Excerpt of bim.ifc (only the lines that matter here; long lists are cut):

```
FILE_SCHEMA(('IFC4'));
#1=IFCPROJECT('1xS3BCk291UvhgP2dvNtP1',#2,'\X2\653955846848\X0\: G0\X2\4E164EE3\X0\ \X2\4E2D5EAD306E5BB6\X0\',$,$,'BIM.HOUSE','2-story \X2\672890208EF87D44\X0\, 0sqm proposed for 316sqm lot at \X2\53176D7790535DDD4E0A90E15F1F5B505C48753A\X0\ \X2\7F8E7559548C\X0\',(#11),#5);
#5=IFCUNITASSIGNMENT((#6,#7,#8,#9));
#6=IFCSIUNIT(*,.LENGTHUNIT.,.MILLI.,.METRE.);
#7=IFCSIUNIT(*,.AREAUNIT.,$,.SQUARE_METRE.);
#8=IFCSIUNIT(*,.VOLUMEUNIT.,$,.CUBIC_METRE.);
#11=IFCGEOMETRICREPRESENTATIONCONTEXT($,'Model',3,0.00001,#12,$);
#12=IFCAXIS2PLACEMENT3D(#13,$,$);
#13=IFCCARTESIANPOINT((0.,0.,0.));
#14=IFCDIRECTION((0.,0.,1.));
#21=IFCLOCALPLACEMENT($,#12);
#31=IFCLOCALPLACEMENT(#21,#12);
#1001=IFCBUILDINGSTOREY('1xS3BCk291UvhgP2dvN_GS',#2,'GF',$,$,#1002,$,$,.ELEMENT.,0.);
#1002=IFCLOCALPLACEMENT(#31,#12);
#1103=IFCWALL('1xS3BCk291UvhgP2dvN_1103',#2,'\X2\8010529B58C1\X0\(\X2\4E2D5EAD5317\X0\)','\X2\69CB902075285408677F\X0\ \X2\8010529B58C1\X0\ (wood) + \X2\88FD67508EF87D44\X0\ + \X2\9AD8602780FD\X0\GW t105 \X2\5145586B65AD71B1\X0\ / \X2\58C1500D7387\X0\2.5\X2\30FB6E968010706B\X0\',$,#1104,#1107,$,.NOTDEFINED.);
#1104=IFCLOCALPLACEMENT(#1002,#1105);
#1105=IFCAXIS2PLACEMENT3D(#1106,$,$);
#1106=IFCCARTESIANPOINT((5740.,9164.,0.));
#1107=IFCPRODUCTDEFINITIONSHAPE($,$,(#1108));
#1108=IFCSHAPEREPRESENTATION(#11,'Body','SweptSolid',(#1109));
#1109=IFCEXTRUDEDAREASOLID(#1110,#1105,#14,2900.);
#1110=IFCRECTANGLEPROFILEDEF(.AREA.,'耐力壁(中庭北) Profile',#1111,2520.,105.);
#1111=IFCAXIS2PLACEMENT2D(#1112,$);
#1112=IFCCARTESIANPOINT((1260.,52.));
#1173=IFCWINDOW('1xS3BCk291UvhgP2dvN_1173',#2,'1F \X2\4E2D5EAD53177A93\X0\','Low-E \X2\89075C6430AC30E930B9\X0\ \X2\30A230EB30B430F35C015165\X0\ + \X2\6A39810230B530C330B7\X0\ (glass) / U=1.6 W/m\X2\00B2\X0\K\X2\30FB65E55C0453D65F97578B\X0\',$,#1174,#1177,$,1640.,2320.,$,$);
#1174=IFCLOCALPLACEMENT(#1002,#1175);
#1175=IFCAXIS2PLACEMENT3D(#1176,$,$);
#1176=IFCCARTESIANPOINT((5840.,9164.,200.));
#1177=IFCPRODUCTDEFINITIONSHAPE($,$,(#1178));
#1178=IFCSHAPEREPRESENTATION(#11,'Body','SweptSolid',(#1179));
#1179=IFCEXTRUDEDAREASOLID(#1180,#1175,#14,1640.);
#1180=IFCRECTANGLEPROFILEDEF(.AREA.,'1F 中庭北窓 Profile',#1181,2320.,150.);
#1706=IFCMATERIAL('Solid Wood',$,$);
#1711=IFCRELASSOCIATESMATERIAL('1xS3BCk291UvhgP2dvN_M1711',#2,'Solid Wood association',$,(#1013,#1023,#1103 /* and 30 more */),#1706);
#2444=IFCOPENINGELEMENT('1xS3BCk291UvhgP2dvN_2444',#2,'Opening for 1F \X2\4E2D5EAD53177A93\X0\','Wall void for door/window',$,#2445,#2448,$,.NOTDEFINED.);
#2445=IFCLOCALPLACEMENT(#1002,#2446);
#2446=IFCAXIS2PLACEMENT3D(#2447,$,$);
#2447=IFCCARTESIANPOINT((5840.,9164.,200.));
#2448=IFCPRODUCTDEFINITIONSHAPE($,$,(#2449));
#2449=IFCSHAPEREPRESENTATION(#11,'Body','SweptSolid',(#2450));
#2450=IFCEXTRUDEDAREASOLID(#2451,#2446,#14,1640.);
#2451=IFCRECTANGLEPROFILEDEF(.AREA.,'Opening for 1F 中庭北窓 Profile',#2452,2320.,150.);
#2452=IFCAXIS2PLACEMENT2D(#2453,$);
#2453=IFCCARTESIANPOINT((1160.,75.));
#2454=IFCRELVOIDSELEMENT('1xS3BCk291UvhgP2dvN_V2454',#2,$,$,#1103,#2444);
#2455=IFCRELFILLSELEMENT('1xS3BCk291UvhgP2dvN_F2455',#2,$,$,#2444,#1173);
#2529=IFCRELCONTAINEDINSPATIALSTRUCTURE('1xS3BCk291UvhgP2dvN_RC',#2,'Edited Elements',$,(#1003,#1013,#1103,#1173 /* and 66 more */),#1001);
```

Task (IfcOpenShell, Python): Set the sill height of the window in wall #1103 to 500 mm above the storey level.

```python
import numpy as np
import ifcopenshell
import ifcopenshell.api.geometry
import ifcopenshell.geom
import ifcopenshell.util.element
import ifcopenshell.util.placement
import ifcopenshell.util.shape
import ifcopenshell.util.unit

model = ifcopenshell.open("bim.ifc")
unit_scale = ifcopenshell.util.unit.calculate_unit_scale(model)

window = model.by_guid("1xS3BCk291UvhgP2dvN_1173")
opening = window.FillsVoids[0].RelatingOpeningElement
storey = ifcopenshell.util.element.get_container(window, ifc_class="IfcBuildingStorey")
level = ifcopenshell.util.placement.get_local_placement(storey.ObjectPlacement)[2, 3]

# The opening's origin need not be at the sill, so measure its lowest point.
shape = ifcopenshell.geom.create_shape(ifcopenshell.geom.settings(), opening)
bottom = ifcopenshell.util.shape.get_shape_bottom_elevation(shape, shape.geometry) / unit_scale
dz = level + 0.5 / unit_scale - bottom

shift = np.array([0.0, 0.0, dz])
# The window is not placed relative to its opening, so move both.
for product in (opening, window):
    matrix = ifcopenshell.util.placement.get_local_placement(product.ObjectPlacement)
    matrix[:3, 3] += shift
    ifcopenshell.api.geometry.edit_object_placement(model, product=product, matrix=matrix, is_si=False)

print(f"moved by {dz * unit_scale:+.3f} m")

model.write("bim_rev.ifc")
```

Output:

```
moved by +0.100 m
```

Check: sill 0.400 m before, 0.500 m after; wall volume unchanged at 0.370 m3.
